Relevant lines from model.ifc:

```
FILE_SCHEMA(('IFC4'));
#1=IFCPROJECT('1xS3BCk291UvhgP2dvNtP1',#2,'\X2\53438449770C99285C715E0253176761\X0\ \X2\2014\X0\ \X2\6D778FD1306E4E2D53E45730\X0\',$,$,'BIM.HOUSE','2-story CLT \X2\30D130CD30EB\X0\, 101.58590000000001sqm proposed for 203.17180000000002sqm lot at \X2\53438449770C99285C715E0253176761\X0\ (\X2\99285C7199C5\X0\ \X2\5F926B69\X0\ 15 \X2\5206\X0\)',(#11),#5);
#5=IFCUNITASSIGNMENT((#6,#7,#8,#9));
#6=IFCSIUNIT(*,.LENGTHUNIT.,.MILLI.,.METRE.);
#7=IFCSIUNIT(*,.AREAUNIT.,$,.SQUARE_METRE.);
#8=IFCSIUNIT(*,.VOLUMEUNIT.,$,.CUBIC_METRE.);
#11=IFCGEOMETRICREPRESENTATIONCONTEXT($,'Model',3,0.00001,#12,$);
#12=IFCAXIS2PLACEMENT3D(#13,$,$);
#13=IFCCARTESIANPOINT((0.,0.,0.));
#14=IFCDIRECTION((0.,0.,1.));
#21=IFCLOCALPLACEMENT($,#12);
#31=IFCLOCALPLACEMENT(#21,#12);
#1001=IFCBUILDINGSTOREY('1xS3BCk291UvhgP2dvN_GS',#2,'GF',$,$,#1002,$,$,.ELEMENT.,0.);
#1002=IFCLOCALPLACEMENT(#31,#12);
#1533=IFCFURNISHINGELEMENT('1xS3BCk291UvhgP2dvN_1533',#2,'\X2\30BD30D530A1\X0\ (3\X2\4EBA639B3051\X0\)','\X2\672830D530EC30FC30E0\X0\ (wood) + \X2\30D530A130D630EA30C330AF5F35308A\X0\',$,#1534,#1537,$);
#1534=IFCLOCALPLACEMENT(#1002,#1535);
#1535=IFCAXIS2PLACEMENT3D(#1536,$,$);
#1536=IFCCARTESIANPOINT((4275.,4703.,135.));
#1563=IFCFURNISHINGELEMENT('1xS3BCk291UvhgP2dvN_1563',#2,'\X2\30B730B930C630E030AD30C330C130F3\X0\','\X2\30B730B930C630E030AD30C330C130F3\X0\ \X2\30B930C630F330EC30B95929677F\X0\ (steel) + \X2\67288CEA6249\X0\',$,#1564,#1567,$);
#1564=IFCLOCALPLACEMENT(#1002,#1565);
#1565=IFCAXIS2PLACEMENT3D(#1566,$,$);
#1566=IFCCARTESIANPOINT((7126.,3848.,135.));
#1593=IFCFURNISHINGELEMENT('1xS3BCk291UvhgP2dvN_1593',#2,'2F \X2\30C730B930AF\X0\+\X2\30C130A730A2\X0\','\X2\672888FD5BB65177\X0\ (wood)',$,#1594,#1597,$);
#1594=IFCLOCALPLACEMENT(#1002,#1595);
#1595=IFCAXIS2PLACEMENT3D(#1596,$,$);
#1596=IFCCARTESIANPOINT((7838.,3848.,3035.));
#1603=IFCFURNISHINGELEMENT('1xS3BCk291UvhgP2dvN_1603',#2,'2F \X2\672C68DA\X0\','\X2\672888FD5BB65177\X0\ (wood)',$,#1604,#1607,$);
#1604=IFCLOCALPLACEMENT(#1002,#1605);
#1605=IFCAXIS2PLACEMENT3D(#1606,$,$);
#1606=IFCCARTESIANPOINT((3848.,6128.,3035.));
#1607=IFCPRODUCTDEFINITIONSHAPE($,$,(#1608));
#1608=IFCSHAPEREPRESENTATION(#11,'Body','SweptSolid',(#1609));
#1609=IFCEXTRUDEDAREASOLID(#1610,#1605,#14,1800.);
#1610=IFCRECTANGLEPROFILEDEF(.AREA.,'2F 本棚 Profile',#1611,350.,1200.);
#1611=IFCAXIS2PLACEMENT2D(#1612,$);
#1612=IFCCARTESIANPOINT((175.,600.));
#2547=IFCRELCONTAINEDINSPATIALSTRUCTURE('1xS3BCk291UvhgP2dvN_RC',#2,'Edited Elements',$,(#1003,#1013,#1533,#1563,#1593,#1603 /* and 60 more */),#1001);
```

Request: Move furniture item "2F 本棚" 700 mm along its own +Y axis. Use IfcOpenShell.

```python
import ifcopenshell
import ifcopenshell.api.geometry
import ifcopenshell.util.placement

model = ifcopenshell.open("model.ifc")

item = model.by_id(1603)
matrix = ifcopenshell.util.placement.get_local_placement(item.ObjectPlacement)
matrix[:3, 3] += matrix[:3, 1] * 700.0
ifcopenshell.api.geometry.edit_object_placement(model, product=item, matrix=matrix, is_si=False)

print(ifcopenshell.util.placement.get_local_placement(item.ObjectPlacement).round(3) + 0.0)

model.write("model_rev.ifc")
```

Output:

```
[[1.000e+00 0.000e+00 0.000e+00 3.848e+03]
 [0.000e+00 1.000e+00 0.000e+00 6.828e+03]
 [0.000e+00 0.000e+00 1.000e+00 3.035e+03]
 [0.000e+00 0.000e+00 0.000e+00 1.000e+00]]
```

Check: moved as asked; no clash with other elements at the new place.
